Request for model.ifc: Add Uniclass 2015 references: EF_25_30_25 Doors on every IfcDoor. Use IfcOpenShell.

First a look at what the model holds.

```python
import ifcopenshell

model = ifcopenshell.open("model.ifc")
print(model.schema)
print("classifications:", [c.Name for c in model.by_type("IfcClassification")])
for ifc_class in ("IfcDoor", "IfcRoof", "IfcStair", "IfcWall", "IfcWindow"):
    print(ifc_class, len(model.by_type(ifc_class)))
```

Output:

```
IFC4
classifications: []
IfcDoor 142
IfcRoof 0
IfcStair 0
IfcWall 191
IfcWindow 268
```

```python
import ifcopenshell
import ifcopenshell.api.classification

model = ifcopenshell.open("model.ifc")

system = ifcopenshell.api.classification.add_classification(model, classification="Uniclass 2015")

codes = {
    "IfcDoor": ("EF_25_30_25", "Doors"),
}
for ifc_class, (code, name) in codes.items():
    products = model.by_type(ifc_class)
    ifcopenshell.api.classification.add_reference(
        model, products=products, classification=system, identification=code, name=name
    )
    print(code, len(products))

model.write("model_edited.ifc")
```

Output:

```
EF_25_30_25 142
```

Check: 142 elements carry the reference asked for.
